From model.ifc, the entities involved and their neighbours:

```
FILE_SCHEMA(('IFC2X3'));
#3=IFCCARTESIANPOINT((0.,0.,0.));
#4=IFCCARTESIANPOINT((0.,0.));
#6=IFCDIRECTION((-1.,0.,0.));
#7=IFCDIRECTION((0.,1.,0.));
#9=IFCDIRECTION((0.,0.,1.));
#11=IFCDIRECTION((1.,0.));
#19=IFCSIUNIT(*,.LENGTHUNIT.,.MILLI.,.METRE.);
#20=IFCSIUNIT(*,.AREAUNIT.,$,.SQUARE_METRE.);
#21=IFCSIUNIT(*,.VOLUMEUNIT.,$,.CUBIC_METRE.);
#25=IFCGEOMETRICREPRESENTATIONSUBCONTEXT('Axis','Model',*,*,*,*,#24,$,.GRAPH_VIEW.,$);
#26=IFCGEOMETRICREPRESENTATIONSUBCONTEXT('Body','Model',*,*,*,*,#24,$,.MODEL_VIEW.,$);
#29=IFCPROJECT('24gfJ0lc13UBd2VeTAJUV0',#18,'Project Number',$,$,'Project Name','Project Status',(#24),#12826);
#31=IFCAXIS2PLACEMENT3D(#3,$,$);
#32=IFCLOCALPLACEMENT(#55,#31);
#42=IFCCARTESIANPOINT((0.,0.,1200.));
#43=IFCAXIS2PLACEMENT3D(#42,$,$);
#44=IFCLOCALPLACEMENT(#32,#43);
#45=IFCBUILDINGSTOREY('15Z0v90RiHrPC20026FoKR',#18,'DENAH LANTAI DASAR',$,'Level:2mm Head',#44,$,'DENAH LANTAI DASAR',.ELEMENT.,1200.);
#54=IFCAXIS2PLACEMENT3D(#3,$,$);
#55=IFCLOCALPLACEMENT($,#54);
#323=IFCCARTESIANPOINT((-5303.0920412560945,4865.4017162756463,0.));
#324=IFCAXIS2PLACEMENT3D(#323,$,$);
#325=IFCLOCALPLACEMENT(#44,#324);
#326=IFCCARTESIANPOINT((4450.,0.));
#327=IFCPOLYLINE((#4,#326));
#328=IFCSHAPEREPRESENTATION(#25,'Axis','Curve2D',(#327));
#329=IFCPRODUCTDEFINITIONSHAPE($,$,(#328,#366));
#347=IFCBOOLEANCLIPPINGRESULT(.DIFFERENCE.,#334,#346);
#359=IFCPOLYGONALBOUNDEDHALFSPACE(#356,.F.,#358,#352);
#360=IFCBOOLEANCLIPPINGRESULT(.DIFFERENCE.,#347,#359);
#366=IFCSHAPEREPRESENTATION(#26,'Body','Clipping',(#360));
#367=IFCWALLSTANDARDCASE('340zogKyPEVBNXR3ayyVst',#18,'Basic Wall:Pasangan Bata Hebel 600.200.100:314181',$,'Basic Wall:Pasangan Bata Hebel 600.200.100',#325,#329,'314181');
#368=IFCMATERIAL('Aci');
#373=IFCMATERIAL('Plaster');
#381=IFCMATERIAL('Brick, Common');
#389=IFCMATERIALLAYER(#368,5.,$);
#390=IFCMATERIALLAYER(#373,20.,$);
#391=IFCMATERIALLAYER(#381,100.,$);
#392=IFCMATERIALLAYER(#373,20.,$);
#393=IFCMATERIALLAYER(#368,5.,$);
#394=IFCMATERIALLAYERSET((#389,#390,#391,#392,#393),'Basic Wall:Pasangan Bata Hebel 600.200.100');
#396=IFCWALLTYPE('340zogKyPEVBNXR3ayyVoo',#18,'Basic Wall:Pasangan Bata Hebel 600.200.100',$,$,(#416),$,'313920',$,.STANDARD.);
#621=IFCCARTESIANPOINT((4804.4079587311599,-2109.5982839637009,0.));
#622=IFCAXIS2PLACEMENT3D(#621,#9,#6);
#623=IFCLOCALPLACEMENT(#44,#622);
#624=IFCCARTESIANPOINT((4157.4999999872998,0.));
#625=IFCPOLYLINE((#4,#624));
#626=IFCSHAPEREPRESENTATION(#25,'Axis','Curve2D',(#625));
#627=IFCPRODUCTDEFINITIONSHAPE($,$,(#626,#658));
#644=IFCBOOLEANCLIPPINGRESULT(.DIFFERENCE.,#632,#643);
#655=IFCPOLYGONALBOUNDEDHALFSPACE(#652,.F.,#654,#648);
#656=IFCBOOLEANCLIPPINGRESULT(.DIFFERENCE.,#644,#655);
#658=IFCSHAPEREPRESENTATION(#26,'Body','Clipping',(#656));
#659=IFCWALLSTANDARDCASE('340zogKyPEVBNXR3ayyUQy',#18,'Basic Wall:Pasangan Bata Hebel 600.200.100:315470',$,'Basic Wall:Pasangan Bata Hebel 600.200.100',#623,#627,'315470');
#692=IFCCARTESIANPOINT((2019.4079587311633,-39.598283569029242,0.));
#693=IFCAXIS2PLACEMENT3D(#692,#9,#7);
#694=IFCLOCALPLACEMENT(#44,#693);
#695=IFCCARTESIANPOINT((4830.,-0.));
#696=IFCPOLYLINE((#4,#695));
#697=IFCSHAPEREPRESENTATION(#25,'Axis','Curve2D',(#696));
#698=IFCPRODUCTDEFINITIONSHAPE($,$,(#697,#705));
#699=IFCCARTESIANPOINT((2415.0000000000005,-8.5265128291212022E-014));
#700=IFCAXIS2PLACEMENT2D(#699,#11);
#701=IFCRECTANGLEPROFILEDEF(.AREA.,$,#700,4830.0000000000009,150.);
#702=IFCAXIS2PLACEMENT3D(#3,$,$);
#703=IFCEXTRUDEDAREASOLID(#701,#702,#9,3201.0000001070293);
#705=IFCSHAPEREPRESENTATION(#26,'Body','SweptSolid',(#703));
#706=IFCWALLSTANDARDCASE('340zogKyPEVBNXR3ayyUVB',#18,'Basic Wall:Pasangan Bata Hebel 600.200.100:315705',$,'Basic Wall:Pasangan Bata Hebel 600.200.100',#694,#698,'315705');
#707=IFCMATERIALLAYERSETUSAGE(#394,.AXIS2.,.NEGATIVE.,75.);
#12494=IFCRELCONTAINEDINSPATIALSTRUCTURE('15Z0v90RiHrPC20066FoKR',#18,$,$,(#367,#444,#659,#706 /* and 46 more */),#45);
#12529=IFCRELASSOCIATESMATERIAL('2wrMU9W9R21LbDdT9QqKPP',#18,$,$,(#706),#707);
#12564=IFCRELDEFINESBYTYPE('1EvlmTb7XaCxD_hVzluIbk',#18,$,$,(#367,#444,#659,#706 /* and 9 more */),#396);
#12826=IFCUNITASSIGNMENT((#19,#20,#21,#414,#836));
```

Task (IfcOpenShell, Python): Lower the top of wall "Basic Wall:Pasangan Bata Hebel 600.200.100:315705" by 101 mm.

```python
import ifcopenshell
import ifcopenshell.geom
import ifcopenshell.util.representation
import ifcopenshell.util.shape

model = ifcopenshell.open("model.ifc")
settings = ifcopenshell.geom.settings()


def volume(element):
    """Net volume in cubic metres, openings subtracted."""
    shape = ifcopenshell.geom.create_shape(settings, element)
    return ifcopenshell.util.shape.get_volume(shape.geometry)


wall = model.by_id(706)
before = volume(wall)

body = ifcopenshell.util.representation.get_representation(wall, "Model", "Body")
solid = body.Items[0]
old_height = solid.Depth
solid.Depth -= 101.0
after = volume(wall)

print(f"height {old_height:g} -> {solid.Depth:g}, volume {before:.3f} -> {after:.3f} m3")

model.write("model-out.ifc")
```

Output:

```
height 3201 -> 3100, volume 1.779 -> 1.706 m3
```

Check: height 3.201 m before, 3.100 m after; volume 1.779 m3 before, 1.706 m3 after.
